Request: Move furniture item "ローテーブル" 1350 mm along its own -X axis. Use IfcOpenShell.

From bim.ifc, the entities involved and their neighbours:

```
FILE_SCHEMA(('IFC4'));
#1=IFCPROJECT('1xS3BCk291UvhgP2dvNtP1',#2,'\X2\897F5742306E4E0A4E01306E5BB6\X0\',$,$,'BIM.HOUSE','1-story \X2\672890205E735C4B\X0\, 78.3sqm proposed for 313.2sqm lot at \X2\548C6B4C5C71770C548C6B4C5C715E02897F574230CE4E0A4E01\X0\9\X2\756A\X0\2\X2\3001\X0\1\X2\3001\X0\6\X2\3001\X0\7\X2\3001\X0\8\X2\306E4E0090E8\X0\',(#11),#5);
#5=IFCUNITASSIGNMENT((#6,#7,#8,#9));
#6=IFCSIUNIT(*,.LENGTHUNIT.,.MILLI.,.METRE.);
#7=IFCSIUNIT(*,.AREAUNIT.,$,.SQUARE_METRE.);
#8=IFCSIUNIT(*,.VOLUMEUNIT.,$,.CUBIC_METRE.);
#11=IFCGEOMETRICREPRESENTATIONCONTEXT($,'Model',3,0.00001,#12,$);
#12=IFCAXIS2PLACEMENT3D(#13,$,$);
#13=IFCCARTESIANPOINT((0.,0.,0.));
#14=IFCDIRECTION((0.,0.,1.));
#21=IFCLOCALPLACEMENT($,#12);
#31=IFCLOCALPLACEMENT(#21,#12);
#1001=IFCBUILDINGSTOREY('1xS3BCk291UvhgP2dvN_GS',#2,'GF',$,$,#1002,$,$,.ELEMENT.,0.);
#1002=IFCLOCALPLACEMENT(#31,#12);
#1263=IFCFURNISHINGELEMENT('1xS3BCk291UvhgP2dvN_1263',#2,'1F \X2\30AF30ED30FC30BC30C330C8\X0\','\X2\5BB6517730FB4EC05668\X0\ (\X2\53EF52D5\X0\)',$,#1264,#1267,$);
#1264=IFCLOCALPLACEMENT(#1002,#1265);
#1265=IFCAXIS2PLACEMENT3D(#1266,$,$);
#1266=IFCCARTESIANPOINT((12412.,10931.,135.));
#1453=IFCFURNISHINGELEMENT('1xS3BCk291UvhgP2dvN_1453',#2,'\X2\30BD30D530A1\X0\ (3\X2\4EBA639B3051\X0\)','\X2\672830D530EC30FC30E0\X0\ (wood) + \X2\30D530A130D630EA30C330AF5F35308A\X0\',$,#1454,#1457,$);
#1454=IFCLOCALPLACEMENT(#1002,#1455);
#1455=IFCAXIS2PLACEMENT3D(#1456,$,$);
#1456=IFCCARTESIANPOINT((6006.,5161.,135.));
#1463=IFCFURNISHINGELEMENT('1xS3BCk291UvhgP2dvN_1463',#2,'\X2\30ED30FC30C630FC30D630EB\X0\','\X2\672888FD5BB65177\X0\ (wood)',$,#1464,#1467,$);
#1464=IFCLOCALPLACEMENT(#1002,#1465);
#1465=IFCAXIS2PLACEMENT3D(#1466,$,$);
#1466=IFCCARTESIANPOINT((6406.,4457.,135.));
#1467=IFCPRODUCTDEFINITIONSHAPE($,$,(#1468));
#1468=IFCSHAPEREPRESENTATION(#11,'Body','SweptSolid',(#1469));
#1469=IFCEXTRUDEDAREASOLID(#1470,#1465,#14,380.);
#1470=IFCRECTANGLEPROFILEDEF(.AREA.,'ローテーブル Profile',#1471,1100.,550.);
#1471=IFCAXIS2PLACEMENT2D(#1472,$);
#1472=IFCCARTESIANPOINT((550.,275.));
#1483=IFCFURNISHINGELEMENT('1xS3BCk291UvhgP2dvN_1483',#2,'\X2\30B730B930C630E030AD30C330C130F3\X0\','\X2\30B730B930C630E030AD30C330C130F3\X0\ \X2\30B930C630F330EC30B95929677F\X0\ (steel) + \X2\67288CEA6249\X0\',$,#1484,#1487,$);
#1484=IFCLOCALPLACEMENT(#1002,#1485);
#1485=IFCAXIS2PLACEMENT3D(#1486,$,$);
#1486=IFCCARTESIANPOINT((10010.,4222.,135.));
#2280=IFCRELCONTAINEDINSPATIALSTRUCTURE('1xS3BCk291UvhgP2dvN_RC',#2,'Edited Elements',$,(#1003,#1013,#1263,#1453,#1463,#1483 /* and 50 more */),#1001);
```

```python
import ifcopenshell
import ifcopenshell.api.geometry
import ifcopenshell.util.placement
import ifcopenshell.util.unit

model = ifcopenshell.open("bim.ifc")
unit_scale = ifcopenshell.util.unit.calculate_unit_scale(model)

item = model.by_id(1463)
matrix = ifcopenshell.util.placement.get_local_placement(item.ObjectPlacement)
matrix[:3, 3] -= matrix[:3, 0] * 1.35 / unit_scale
ifcopenshell.api.geometry.edit_object_placement(model, product=item, matrix=matrix, is_si=False)

print(ifcopenshell.util.placement.get_local_placement(item.ObjectPlacement).round(3) + 0.0)

model.write("bim-out.ifc")
```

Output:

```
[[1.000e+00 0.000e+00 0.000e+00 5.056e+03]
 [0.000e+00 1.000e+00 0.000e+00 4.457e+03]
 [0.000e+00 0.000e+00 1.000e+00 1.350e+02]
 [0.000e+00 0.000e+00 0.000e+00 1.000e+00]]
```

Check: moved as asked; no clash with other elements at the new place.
